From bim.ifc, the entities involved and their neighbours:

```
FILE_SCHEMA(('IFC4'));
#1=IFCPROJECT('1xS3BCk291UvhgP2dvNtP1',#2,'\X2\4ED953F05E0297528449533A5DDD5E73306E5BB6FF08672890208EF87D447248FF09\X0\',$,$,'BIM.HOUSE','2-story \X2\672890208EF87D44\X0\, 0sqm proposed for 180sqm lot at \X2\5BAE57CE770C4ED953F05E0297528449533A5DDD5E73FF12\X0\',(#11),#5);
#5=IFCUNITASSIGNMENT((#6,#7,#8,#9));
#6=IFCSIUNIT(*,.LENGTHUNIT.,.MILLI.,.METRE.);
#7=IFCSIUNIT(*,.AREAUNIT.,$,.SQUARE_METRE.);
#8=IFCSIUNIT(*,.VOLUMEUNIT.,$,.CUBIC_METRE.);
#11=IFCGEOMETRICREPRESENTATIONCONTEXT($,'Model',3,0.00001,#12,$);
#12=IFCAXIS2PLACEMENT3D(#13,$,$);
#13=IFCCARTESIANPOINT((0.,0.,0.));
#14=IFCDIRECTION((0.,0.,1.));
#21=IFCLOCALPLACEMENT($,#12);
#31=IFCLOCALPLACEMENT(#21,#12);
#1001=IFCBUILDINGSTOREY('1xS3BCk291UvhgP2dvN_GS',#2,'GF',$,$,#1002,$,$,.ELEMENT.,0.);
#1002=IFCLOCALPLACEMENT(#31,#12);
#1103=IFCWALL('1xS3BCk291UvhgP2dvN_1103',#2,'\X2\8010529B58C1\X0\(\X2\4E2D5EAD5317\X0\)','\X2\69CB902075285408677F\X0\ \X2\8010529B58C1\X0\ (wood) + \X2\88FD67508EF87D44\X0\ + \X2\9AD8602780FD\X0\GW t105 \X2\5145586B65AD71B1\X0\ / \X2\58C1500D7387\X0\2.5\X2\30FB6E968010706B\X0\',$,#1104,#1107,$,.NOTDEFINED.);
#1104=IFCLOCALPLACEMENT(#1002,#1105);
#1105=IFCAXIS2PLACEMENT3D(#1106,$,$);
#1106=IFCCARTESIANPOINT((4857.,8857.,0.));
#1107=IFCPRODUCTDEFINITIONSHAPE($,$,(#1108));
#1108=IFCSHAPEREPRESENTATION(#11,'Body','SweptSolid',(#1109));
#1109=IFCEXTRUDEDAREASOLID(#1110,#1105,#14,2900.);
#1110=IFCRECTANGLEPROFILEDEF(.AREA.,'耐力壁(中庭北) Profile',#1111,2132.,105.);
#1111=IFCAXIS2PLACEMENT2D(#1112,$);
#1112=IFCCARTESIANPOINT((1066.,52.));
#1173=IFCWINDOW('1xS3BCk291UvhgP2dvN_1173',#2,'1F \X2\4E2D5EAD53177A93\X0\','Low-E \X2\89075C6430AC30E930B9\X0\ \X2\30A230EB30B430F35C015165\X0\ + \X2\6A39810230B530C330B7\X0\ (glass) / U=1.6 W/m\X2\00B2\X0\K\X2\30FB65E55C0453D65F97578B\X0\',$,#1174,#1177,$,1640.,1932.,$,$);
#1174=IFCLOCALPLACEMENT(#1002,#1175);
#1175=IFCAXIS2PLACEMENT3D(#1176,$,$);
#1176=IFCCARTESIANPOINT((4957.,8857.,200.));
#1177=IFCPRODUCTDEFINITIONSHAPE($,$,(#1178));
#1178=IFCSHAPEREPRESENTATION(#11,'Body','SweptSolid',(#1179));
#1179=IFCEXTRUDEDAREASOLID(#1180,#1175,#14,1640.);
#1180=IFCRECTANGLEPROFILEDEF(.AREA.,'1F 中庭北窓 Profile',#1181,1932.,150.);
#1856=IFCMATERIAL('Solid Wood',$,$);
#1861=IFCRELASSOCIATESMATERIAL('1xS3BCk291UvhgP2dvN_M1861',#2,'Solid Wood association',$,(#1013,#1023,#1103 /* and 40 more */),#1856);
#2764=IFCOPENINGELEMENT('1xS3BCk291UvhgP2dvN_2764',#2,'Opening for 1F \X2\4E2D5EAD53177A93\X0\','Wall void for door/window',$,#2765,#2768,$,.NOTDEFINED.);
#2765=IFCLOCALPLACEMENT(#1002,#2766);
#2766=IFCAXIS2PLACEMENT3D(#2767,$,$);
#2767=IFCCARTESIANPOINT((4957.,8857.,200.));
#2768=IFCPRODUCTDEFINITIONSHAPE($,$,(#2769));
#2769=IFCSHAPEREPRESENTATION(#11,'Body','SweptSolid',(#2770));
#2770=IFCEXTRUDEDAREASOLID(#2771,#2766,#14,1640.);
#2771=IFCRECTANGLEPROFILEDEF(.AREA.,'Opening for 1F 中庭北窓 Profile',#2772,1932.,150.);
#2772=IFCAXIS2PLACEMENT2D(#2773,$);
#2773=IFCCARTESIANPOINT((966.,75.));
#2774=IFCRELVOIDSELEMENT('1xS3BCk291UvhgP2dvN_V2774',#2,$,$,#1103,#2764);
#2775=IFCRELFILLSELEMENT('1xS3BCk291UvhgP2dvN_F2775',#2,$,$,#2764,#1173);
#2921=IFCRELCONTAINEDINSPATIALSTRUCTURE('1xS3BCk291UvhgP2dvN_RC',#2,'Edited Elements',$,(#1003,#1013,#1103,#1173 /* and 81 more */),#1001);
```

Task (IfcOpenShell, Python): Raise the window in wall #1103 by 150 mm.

```python
import numpy as np
import ifcopenshell
import ifcopenshell.api.geometry
import ifcopenshell.util.placement
import ifcopenshell.util.unit

model = ifcopenshell.open("bim.ifc")
unit_scale = ifcopenshell.util.unit.calculate_unit_scale(model)

window = model.by_id(1173)
opening = window.FillsVoids[0].RelatingOpeningElement
dz = 150.0

shift = np.array([0.0, 0.0, dz])
# The window is not placed relative to its opening, so move both.
for product in (opening, window):
    matrix = ifcopenshell.util.placement.get_local_placement(product.ObjectPlacement)
    matrix[:3, 3] += shift
    ifcopenshell.api.geometry.edit_object_placement(model, product=product, matrix=matrix, is_si=False)

print(f"moved by {dz * unit_scale:+.3f} m")

model.write("bim-out.ifc")
```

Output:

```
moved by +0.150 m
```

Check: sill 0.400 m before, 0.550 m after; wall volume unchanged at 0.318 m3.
